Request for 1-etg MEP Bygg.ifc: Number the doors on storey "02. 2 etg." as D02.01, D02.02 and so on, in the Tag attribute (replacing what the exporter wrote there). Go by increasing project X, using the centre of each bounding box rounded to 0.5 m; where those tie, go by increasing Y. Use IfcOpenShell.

First a look at what the model holds.

```python
import ifcopenshell
import ifcopenshell.util.element
import ifcopenshell.util.placement

model = ifcopenshell.open("1-etg MEP Bygg.ifc")
print(model.schema)
storey = next(s for s in model.by_type("IfcBuildingStorey") if s.Name == "02. 2 etg.")
doors = [e for e in ifcopenshell.util.element.get_decomposition(storey) if e.is_a("IfcDoor")]
for e in sorted(doors, key=lambda e: e.id()):
    origin = ifcopenshell.util.placement.get_local_placement(e.ObjectPlacement)[:3, 3]
    print(e.id(), e.Tag, e.Name, origin.round(2) + 0.0, sep=" | ")
```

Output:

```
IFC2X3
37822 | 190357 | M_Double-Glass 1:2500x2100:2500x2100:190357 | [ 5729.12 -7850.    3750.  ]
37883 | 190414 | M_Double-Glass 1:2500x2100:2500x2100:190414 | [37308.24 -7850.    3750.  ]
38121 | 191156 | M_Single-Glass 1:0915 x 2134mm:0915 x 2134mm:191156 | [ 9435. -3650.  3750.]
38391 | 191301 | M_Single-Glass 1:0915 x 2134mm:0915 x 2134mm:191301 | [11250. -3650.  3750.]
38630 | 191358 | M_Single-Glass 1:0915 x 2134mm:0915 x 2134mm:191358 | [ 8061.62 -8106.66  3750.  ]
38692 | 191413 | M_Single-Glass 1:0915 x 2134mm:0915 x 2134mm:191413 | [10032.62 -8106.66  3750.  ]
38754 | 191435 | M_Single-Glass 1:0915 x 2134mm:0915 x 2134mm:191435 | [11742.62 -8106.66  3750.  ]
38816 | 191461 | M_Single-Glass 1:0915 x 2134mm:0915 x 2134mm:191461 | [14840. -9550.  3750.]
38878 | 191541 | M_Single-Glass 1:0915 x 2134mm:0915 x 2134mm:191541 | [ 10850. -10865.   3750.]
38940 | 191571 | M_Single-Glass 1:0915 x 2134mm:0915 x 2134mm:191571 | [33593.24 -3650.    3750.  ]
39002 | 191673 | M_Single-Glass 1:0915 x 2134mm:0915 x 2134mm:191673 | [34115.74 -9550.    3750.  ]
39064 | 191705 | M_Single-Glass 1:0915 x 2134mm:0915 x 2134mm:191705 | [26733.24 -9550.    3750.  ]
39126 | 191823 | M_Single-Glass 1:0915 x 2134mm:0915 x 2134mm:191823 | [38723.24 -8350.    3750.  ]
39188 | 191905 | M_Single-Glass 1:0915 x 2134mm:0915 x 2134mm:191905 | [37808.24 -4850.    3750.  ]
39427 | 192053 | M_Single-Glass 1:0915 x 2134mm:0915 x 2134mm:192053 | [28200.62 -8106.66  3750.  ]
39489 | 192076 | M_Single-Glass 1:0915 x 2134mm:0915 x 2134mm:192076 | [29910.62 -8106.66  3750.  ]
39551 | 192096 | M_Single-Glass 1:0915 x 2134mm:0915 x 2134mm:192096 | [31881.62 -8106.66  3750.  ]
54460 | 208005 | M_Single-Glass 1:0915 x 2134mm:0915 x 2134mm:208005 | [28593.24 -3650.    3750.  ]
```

```python
import ifcopenshell
import ifcopenshell.geom
import ifcopenshell.util.element
import ifcopenshell.util.shape

model = ifcopenshell.open("1-etg MEP Bygg.ifc")
settings = ifcopenshell.geom.settings()
settings.set("use-world-coords", True)


def centre(element):
    shape = ifcopenshell.geom.create_shape(settings, element)
    return ifcopenshell.util.shape.get_bbox_centroid(shape.geometry)


storey = next(s for s in model.by_type("IfcBuildingStorey") if s.Name == "02. 2 etg.")
doors = [e for e in ifcopenshell.util.element.get_decomposition(storey) if e.is_a("IfcDoor")]

# Insertion points can sit at a corner or the storey origin, so sort by the geometry (in metres).
centres = {e: centre(e) for e in doors}
doors.sort(key=lambda e: (round(centres[e][0] / 0.5), centres[e][1]))

for i, e in enumerate(doors, start=1):
    number = f"D02.{i:02d}"
    e.Tag = number
    print(e.id(), number)

model.write("1-etg MEP Bygg_updated.ifc")
```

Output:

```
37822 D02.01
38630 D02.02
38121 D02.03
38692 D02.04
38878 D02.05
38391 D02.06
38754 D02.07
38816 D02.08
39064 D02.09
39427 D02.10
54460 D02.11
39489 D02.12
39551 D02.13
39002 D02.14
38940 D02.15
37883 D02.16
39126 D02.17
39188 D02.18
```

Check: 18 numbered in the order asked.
